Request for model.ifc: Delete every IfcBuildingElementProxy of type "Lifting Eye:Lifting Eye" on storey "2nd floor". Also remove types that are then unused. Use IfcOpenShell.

First a look at what the model holds.

```python
import ifcopenshell
import ifcopenshell.util.element

model = ifcopenshell.open("model.ifc")
print(model.schema)
storey = next(s for s in model.by_type("IfcBuildingStorey") if s.Name == "2nd floor")
proxies = [e for e in ifcopenshell.util.element.get_decomposition(storey) if e.is_a("IfcBuildingElementProxy")]
seen = {}
for e in proxies:
    element_type = ifcopenshell.util.element.get_type(e)
    name = element_type.Name if element_type not in (None, e) else None
    seen[name] = seen.get(name, 0) + 1
for name, count in sorted(seen.items(), key=str):
    print(count, "x", name)
```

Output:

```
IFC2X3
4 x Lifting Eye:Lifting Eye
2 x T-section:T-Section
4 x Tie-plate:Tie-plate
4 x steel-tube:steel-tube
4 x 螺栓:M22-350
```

```python
import ifcopenshell
import ifcopenshell.api.root
import ifcopenshell.util.element

model = ifcopenshell.open("model.ifc")

storey = next(s for s in model.by_type("IfcBuildingStorey") if s.Name == "2nd floor")
proxies = [e for e in ifcopenshell.util.element.get_decomposition(storey) if e.is_a("IfcBuildingElementProxy")]
targets = [e for e in proxies if (t := ifcopenshell.util.element.get_type(e)) not in (None, e) and t.Name == "Lifting Eye:Lifting Eye"]
types = {ifcopenshell.util.element.get_type(e) for e in targets} - {None, *targets}

for e in targets:
    ifcopenshell.api.root.remove_product(model, product=e)
print(len(targets), "removed")

unused = [t for t in types if not ifcopenshell.util.element.get_types(t)]
for t in unused:
    ifcopenshell.api.root.remove_product(model, product=t)
print(len(unused), "unused types removed")

model.write("model_rev.ifc")
```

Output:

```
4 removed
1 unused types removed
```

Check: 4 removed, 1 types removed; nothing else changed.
